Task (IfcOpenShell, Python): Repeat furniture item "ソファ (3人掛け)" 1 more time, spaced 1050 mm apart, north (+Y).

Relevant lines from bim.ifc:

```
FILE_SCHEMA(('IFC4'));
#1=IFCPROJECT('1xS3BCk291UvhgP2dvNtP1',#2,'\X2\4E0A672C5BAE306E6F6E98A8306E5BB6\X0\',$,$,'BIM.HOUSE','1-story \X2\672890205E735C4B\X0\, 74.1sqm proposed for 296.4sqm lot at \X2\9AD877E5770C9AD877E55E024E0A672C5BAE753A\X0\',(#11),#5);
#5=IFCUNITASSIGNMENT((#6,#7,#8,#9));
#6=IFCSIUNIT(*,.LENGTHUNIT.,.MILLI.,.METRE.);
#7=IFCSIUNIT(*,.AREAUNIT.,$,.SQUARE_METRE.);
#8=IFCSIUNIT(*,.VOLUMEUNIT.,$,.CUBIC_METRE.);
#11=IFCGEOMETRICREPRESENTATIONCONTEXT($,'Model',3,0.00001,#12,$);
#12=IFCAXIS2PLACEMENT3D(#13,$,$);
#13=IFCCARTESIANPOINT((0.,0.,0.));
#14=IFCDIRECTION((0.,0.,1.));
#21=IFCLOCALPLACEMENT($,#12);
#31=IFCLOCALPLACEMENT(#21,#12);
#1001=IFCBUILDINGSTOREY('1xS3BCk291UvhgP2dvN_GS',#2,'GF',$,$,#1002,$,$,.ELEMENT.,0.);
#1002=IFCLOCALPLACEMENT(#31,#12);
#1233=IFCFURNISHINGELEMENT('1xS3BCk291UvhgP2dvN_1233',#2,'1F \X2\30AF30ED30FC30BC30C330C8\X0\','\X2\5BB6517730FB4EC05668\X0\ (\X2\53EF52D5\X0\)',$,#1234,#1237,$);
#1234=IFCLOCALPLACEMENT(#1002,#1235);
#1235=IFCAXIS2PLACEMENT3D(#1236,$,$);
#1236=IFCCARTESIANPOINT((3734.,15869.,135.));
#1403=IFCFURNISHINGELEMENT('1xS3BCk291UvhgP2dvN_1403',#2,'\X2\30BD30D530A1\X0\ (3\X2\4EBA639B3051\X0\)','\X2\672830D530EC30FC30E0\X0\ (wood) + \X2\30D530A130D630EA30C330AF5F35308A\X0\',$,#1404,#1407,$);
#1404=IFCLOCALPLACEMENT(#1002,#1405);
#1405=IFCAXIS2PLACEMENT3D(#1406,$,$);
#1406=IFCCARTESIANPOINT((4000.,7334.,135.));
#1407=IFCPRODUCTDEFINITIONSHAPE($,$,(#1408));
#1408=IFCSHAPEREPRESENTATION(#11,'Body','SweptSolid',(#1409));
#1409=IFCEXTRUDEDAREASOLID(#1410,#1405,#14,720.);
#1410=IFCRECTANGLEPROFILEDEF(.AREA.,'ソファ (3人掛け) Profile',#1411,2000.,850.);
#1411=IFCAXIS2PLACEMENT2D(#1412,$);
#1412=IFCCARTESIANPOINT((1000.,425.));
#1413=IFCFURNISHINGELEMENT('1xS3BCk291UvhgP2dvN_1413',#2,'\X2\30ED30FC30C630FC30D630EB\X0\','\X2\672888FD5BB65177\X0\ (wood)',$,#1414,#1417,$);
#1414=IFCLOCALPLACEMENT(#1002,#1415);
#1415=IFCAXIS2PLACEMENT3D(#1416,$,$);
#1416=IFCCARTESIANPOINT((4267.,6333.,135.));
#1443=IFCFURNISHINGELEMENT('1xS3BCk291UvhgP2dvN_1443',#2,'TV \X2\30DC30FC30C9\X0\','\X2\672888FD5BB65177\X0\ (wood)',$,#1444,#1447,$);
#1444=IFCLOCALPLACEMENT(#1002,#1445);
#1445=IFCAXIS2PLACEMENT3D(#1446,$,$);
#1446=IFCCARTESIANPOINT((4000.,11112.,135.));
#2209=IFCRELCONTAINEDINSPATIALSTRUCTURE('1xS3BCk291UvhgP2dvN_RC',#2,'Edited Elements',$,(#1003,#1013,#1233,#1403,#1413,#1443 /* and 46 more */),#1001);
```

```python
import numpy as np
import ifcopenshell
import ifcopenshell.api.geometry
import ifcopenshell.api.root
import ifcopenshell.util.element
import ifcopenshell.util.placement

model = ifcopenshell.open("bim.ifc")


def reuse_history(source, copy):
    """copy_class also copies each property set's owner history, people and application; keep the originals."""
    for rel in copy.IsDefinedBy:
        if rel.is_a("IfcRelDefinesByProperties") and (history := rel.RelatingPropertyDefinition.OwnerHistory):
            rel.RelatingPropertyDefinition.OwnerHistory = source.OwnerHistory
            ifcopenshell.util.element.remove_deep2(model, history)


source = model.by_guid("1xS3BCk291UvhgP2dvN_1403")
base = ifcopenshell.util.placement.get_local_placement(source.ObjectPlacement)
step = np.array([0.0, 1.0, 0.0]) * 1050.0

for i in range(1, 2):
    copy = ifcopenshell.api.root.copy_class(model, product=source)
    copy.Representation = ifcopenshell.util.element.copy_deep(
        model, source.Representation, exclude=["IfcGeometricRepresentationContext", "IfcRepresentationMap"]
    )
    reuse_history(source, copy)
    matrix = base.copy()
    matrix[:3, 3] += i * step
    print("added at", matrix[:3, 3].round(3) + 0.0)
    ifcopenshell.api.geometry.edit_object_placement(model, product=copy, matrix=matrix, is_si=False)

model.write("bim_v2.ifc")
```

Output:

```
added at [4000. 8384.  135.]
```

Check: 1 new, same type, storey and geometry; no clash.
